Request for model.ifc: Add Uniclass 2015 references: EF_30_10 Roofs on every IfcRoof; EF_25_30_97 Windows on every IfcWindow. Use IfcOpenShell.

First a look at what the model holds.

```python
import ifcopenshell

model = ifcopenshell.open("model.ifc")
print(model.schema)
print("classifications:", [c.Name for c in model.by_type("IfcClassification")])
for ifc_class in ("IfcDoor", "IfcRoof", "IfcStair", "IfcWall", "IfcWindow"):
    print(ifc_class, len(model.by_type(ifc_class)))
```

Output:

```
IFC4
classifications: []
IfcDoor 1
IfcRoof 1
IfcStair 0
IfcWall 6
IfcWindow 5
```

```python
import ifcopenshell
import ifcopenshell.api.classification

model = ifcopenshell.open("model.ifc")

system = ifcopenshell.api.classification.add_classification(model, classification="Uniclass 2015")

codes = {
    "IfcRoof": ("EF_30_10", "Roofs"),
    "IfcWindow": ("EF_25_30_97", "Windows"),
}
for ifc_class, (code, name) in codes.items():
    products = model.by_type(ifc_class)
    ifcopenshell.api.classification.add_reference(
        model, products=products, classification=system, identification=code, name=name
    )
    print(code, len(products))

model.write("model_edited.ifc")
```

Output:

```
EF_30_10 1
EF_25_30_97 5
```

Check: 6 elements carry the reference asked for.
